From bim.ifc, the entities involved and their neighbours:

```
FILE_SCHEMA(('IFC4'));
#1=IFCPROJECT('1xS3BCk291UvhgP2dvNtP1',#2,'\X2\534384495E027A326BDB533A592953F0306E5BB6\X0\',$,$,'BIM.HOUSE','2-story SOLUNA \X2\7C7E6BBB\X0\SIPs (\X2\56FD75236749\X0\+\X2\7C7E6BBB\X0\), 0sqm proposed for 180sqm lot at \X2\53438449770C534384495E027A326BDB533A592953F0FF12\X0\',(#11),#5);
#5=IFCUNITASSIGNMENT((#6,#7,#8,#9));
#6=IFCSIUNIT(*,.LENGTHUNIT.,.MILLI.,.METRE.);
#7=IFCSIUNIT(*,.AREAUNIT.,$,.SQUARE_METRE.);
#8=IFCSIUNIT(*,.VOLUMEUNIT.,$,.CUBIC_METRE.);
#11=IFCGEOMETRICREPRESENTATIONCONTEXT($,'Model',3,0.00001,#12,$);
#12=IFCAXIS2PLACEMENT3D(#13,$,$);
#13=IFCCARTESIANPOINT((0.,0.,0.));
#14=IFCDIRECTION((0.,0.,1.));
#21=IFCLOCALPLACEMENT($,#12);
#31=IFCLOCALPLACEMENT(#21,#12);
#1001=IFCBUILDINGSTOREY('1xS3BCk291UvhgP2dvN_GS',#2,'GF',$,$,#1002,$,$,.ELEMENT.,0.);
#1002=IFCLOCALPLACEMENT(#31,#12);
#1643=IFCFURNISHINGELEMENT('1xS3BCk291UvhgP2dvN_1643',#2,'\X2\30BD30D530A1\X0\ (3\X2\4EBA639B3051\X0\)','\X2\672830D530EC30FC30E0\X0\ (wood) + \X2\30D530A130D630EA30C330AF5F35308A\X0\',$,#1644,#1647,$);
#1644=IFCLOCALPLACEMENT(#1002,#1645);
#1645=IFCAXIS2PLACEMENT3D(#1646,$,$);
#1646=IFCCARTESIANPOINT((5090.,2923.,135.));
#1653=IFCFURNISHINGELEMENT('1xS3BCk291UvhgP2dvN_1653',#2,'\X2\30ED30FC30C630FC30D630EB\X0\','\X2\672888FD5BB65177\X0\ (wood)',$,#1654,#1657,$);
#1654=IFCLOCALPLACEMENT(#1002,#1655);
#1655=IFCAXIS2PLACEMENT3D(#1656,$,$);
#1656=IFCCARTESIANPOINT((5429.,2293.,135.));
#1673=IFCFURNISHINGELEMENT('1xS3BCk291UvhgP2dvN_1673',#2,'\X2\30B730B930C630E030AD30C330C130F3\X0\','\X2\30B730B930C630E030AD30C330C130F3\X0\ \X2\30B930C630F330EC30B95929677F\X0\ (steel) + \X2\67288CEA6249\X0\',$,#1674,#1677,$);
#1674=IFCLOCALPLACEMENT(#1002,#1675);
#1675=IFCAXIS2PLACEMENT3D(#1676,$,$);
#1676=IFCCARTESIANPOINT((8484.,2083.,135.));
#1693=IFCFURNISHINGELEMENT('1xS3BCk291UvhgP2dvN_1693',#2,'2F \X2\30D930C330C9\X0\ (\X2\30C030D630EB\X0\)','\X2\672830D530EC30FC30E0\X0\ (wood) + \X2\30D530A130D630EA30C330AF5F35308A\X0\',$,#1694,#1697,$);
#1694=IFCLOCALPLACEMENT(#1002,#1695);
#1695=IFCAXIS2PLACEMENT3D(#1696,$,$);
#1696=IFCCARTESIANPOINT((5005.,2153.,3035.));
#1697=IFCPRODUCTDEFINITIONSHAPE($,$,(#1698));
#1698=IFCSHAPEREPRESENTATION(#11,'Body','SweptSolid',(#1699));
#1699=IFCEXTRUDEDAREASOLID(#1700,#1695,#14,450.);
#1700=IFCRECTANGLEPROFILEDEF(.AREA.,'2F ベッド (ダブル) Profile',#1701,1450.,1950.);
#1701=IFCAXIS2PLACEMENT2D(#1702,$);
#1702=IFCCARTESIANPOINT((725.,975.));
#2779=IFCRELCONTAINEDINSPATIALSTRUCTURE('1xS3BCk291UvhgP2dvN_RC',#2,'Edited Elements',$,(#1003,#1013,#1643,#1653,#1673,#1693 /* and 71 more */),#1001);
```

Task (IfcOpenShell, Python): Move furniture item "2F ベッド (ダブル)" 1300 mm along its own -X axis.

```python
import ifcopenshell
import ifcopenshell.api.geometry
import ifcopenshell.util.placement

model = ifcopenshell.open("bim.ifc")

item = model.by_guid("1xS3BCk291UvhgP2dvN_1693")
matrix = ifcopenshell.util.placement.get_local_placement(item.ObjectPlacement)
matrix[:3, 3] -= matrix[:3, 0] * 1300.0
ifcopenshell.api.geometry.edit_object_placement(model, product=item, matrix=matrix, is_si=False)

print(ifcopenshell.util.placement.get_local_placement(item.ObjectPlacement).round(3) + 0.0)

model.write("bim_edited.ifc")
```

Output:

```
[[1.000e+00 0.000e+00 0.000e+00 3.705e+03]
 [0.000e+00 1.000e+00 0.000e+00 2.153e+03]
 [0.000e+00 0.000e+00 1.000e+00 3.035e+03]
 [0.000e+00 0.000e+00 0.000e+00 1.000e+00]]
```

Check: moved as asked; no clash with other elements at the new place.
